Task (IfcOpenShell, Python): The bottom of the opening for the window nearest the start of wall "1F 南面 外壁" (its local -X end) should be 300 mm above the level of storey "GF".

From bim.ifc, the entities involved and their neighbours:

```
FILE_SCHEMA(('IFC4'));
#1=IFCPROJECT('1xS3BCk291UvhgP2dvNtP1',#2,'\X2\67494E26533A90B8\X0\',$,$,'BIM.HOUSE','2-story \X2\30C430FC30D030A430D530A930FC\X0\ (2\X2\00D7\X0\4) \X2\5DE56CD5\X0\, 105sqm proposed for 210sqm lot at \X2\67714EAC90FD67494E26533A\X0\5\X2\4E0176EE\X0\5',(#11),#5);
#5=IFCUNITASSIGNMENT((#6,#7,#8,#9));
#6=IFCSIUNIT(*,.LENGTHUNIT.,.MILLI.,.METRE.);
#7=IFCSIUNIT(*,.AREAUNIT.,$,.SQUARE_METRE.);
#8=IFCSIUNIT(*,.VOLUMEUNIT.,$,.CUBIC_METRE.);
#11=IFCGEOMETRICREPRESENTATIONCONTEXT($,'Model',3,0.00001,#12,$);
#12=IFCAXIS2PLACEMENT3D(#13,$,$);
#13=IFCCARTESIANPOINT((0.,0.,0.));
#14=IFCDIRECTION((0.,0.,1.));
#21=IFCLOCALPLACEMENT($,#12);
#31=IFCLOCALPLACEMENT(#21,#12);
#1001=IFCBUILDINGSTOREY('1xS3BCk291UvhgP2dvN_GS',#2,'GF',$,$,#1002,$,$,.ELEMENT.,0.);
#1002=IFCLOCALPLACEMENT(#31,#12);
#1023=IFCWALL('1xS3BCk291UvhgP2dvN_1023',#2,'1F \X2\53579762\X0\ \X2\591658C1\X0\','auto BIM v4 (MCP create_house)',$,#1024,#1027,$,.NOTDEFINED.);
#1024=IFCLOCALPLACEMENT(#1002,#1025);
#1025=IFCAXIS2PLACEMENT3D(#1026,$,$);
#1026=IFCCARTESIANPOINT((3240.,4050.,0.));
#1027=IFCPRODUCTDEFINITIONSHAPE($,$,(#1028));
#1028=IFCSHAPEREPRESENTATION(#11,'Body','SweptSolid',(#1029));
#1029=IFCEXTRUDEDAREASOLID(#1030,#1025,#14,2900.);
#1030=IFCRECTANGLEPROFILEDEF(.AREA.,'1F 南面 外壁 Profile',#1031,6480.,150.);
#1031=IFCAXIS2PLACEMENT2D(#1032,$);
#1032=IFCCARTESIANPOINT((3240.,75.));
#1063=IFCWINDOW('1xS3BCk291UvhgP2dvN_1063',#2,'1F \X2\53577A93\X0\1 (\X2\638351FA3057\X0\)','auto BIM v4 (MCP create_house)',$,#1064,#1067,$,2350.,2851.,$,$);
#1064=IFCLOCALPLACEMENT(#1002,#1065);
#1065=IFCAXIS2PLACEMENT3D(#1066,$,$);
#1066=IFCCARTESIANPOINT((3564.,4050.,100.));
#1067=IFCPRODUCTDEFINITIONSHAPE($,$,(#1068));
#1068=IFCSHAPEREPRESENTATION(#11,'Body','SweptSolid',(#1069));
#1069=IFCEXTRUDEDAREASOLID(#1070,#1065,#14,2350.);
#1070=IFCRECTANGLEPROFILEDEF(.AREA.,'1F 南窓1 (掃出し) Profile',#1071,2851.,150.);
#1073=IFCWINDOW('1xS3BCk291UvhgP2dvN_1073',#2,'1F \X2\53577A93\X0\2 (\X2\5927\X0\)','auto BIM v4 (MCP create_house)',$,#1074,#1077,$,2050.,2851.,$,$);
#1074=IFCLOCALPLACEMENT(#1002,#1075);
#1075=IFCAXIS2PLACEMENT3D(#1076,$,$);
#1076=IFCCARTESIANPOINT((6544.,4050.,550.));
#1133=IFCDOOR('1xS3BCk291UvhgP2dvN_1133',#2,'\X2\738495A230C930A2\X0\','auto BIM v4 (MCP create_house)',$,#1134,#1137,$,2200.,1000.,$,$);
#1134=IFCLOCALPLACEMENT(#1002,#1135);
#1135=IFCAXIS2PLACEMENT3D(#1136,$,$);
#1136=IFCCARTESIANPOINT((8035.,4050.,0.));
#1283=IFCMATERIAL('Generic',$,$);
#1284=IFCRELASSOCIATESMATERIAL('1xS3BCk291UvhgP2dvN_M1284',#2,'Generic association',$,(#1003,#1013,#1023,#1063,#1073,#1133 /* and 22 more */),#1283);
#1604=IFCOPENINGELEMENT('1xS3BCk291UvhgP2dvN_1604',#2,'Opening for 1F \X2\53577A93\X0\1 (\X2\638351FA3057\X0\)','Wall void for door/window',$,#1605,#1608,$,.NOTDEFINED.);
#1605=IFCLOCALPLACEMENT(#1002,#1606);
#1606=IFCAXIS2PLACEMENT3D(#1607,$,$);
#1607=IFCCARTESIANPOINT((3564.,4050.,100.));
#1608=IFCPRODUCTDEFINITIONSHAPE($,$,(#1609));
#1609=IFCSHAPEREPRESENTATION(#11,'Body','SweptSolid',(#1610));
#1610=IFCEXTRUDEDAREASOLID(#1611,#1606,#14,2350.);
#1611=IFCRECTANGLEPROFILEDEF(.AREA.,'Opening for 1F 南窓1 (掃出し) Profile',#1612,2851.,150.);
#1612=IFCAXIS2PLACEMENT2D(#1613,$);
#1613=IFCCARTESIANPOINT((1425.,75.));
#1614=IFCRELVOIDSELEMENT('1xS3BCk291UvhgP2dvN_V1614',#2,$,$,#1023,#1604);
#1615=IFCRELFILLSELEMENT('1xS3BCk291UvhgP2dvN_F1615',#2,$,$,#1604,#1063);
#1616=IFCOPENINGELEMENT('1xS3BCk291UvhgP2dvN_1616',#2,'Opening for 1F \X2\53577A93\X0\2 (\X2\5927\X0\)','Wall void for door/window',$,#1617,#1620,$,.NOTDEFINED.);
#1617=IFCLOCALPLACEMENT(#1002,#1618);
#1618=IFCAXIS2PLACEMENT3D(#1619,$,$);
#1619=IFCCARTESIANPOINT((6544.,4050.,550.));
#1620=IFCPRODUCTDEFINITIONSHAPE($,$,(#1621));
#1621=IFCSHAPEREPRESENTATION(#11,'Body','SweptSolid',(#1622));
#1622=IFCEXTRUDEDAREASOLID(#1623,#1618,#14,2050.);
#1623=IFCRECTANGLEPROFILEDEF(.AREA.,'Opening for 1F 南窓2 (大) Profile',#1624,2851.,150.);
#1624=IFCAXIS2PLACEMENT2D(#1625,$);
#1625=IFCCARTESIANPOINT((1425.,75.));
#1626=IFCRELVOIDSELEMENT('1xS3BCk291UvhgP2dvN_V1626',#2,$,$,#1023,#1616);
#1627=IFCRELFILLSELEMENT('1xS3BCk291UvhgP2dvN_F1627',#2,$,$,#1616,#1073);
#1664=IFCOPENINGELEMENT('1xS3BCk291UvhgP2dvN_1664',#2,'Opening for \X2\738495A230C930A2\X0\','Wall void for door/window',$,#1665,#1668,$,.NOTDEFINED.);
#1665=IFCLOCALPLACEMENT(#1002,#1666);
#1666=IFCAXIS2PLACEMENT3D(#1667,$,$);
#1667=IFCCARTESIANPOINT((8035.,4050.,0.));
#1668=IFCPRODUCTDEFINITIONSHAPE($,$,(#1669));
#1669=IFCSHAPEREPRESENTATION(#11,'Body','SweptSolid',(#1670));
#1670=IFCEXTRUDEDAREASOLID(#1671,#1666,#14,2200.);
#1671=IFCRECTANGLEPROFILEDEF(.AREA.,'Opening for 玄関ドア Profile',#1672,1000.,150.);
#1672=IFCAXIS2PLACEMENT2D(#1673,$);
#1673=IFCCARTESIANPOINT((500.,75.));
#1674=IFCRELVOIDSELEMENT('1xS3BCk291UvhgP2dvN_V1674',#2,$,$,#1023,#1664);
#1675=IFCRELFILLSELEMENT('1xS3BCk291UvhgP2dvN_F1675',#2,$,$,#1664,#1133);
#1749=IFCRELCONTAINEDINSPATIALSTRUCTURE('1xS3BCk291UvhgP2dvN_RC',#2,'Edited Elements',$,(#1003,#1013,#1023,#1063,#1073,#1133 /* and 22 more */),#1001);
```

```python
import numpy as np
import ifcopenshell
import ifcopenshell.api.geometry
import ifcopenshell.geom
import ifcopenshell.util.element
import ifcopenshell.util.placement
import ifcopenshell.util.shape
import ifcopenshell.util.unit

model = ifcopenshell.open("bim.ifc")
unit_scale = ifcopenshell.util.unit.calculate_unit_scale(model)

window = model.by_guid("1xS3BCk291UvhgP2dvN_1063")
opening = window.FillsVoids[0].RelatingOpeningElement
storey = ifcopenshell.util.element.get_container(window, ifc_class="IfcBuildingStorey")
level = ifcopenshell.util.placement.get_local_placement(storey.ObjectPlacement)[2, 3]

# The opening's origin need not be at the sill, so measure its lowest point.
shape = ifcopenshell.geom.create_shape(ifcopenshell.geom.settings(), opening)
bottom = ifcopenshell.util.shape.get_shape_bottom_elevation(shape, shape.geometry) / unit_scale
dz = level + 0.3 / unit_scale - bottom

shift = np.array([0.0, 0.0, dz])
# The window is not placed relative to its opening, so move both.
for product in (opening, window):
    matrix = ifcopenshell.util.placement.get_local_placement(product.ObjectPlacement)
    matrix[:3, 3] += shift
    ifcopenshell.api.geometry.edit_object_placement(model, product=product, matrix=matrix, is_si=False)

print(f"moved by {dz * unit_scale:+.3f} m")

model.write("bim-out.ifc")
```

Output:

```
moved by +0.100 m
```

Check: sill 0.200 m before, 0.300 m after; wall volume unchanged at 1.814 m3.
